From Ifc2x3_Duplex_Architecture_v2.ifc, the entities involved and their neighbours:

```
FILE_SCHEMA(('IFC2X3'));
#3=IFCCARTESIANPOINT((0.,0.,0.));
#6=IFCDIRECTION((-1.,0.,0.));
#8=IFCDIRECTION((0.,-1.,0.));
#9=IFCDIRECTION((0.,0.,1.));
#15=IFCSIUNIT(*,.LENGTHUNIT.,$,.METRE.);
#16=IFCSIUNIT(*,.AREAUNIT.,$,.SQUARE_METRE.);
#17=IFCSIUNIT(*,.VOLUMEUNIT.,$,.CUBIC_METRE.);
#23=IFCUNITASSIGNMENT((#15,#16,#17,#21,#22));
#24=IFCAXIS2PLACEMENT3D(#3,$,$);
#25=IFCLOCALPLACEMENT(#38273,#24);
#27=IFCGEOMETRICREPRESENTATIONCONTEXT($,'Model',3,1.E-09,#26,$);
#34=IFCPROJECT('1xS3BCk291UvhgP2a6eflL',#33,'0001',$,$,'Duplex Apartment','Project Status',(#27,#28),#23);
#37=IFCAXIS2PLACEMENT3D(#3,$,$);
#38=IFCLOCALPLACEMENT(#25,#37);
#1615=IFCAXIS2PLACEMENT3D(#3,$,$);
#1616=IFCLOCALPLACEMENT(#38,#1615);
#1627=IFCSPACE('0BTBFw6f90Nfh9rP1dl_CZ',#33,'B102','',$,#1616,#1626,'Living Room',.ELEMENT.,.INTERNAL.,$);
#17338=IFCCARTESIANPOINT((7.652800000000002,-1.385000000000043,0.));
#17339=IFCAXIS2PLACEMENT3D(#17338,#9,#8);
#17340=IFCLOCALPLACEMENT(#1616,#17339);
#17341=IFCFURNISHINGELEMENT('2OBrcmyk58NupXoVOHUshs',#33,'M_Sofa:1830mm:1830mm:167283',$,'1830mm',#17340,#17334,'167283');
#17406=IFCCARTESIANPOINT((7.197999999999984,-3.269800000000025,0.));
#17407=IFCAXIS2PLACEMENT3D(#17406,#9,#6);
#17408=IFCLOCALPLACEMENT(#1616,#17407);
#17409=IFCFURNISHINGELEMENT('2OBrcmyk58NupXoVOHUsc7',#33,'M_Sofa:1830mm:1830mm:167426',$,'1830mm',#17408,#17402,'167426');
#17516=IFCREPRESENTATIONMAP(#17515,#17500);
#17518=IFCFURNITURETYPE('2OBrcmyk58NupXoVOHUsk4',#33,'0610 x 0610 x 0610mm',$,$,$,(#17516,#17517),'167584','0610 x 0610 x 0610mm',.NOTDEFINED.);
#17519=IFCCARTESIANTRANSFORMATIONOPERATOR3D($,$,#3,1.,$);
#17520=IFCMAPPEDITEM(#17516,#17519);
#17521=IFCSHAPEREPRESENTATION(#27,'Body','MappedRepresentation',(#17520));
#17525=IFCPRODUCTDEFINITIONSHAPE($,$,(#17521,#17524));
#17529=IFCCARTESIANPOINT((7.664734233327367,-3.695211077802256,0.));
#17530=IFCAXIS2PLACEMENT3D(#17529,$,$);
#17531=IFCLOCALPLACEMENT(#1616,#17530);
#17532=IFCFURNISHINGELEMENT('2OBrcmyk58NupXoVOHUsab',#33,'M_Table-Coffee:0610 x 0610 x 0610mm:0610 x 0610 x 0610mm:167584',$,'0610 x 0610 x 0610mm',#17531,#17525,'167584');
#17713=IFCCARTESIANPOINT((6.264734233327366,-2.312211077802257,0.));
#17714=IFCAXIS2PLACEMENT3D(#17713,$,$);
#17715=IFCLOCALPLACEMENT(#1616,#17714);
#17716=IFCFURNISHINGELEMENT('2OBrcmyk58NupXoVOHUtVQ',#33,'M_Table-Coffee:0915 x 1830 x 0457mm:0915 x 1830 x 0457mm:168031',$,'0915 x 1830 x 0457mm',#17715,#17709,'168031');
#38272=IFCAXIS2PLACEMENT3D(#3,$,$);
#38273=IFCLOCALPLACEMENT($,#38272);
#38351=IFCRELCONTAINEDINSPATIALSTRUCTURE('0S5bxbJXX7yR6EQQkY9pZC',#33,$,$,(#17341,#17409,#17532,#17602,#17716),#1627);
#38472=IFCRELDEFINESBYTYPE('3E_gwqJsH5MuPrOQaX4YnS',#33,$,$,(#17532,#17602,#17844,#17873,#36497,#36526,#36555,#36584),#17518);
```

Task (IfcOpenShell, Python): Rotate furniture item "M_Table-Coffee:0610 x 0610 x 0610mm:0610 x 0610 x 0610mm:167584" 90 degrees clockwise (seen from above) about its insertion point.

```python
import ifcopenshell
import ifcopenshell.api.geometry
import ifcopenshell.util.placement

model = ifcopenshell.open("Ifc2x3_Duplex_Architecture_v2.ifc")

item = model.by_id(17532)
matrix = ifcopenshell.util.placement.get_local_placement(item.ObjectPlacement)
matrix = matrix @ ifcopenshell.util.placement.rotation(-90, "Z")
ifcopenshell.api.geometry.edit_object_placement(model, product=item, matrix=matrix, is_si=False)

print(ifcopenshell.util.placement.get_local_placement(item.ObjectPlacement).round(3) + 0.0)

model.write("Ifc2x3_Duplex_Architecture_v2_edited.ifc")
```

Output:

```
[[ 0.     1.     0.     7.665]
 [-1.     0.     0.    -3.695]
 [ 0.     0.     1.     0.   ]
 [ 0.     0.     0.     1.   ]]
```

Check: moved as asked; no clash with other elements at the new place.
